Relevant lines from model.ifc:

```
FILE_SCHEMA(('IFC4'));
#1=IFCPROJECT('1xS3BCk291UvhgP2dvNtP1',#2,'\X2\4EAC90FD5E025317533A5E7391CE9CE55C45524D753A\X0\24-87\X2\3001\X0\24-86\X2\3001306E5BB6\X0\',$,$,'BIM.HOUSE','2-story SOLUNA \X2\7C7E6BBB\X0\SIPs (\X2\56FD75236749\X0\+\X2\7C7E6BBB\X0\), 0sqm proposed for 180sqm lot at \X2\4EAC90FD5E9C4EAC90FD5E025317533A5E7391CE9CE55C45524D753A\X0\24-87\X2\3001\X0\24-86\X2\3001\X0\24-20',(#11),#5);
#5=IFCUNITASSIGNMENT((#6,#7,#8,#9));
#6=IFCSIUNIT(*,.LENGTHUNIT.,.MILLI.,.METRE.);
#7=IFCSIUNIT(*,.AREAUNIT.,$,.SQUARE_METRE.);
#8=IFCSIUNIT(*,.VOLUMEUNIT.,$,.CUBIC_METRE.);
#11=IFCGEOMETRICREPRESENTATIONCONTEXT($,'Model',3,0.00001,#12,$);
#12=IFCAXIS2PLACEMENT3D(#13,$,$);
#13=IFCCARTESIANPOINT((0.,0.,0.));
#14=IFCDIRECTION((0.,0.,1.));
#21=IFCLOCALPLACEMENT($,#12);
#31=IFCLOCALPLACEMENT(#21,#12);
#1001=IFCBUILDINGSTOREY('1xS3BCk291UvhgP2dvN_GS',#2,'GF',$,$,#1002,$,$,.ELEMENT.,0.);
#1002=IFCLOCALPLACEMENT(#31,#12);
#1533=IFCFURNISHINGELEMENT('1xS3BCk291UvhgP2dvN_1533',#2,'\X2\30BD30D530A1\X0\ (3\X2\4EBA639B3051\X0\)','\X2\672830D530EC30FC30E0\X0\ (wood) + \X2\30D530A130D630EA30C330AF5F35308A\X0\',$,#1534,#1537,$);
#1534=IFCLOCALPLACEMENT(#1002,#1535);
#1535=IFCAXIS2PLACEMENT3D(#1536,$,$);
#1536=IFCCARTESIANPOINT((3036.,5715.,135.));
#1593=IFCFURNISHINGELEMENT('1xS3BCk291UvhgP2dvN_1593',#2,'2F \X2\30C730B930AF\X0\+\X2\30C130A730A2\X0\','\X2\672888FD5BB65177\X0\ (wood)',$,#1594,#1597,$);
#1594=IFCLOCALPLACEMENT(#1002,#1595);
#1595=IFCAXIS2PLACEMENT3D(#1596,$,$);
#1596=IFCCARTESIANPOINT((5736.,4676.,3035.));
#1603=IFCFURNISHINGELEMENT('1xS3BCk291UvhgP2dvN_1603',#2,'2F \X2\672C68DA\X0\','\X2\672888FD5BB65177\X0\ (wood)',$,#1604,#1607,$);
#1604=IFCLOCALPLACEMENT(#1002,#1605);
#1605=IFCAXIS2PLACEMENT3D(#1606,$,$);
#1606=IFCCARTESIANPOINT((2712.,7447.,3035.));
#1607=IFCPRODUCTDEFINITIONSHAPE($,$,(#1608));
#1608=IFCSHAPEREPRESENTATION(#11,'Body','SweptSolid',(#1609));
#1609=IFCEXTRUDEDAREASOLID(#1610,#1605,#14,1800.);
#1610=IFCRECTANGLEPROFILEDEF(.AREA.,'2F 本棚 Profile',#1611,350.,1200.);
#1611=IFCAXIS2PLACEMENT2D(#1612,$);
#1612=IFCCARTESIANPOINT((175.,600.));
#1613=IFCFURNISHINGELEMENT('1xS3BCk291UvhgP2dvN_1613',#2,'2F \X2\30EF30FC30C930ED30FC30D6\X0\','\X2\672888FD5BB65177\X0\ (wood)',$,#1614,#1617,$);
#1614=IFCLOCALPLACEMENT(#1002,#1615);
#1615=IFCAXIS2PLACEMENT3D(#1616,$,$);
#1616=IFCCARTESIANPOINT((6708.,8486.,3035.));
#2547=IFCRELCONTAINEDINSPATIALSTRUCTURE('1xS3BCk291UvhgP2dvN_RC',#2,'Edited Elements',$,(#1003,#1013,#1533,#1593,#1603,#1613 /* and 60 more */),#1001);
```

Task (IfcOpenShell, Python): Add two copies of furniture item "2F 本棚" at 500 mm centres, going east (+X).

```python
import numpy as np
import ifcopenshell
import ifcopenshell.api.geometry
import ifcopenshell.api.root
import ifcopenshell.util.element
import ifcopenshell.util.placement
import ifcopenshell.util.unit

model = ifcopenshell.open("model.ifc")
unit_scale = ifcopenshell.util.unit.calculate_unit_scale(model)


def reuse_history(source, copy):
    """copy_class also copies each property set's owner history, people and application; keep the originals."""
    for rel in copy.IsDefinedBy:
        if rel.is_a("IfcRelDefinesByProperties") and (history := rel.RelatingPropertyDefinition.OwnerHistory):
            rel.RelatingPropertyDefinition.OwnerHistory = source.OwnerHistory
            ifcopenshell.util.element.remove_deep2(model, history)


source = model.by_guid("1xS3BCk291UvhgP2dvN_1603")
base = ifcopenshell.util.placement.get_local_placement(source.ObjectPlacement)
step = np.array([1.0, 0.0, 0.0]) * 0.5 / unit_scale

for i in range(1, 3):
    copy = ifcopenshell.api.root.copy_class(model, product=source)
    copy.Representation = ifcopenshell.util.element.copy_deep(
        model, source.Representation, exclude=["IfcGeometricRepresentationContext", "IfcRepresentationMap"]
    )
    reuse_history(source, copy)
    matrix = base.copy()
    matrix[:3, 3] += i * step
    print("added at", matrix[:3, 3].round(3) + 0.0)
    ifcopenshell.api.geometry.edit_object_placement(model, product=copy, matrix=matrix, is_si=False)

model.write("model_v2.ifc")
```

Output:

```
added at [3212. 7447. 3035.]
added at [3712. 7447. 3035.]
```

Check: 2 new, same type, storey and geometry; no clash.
